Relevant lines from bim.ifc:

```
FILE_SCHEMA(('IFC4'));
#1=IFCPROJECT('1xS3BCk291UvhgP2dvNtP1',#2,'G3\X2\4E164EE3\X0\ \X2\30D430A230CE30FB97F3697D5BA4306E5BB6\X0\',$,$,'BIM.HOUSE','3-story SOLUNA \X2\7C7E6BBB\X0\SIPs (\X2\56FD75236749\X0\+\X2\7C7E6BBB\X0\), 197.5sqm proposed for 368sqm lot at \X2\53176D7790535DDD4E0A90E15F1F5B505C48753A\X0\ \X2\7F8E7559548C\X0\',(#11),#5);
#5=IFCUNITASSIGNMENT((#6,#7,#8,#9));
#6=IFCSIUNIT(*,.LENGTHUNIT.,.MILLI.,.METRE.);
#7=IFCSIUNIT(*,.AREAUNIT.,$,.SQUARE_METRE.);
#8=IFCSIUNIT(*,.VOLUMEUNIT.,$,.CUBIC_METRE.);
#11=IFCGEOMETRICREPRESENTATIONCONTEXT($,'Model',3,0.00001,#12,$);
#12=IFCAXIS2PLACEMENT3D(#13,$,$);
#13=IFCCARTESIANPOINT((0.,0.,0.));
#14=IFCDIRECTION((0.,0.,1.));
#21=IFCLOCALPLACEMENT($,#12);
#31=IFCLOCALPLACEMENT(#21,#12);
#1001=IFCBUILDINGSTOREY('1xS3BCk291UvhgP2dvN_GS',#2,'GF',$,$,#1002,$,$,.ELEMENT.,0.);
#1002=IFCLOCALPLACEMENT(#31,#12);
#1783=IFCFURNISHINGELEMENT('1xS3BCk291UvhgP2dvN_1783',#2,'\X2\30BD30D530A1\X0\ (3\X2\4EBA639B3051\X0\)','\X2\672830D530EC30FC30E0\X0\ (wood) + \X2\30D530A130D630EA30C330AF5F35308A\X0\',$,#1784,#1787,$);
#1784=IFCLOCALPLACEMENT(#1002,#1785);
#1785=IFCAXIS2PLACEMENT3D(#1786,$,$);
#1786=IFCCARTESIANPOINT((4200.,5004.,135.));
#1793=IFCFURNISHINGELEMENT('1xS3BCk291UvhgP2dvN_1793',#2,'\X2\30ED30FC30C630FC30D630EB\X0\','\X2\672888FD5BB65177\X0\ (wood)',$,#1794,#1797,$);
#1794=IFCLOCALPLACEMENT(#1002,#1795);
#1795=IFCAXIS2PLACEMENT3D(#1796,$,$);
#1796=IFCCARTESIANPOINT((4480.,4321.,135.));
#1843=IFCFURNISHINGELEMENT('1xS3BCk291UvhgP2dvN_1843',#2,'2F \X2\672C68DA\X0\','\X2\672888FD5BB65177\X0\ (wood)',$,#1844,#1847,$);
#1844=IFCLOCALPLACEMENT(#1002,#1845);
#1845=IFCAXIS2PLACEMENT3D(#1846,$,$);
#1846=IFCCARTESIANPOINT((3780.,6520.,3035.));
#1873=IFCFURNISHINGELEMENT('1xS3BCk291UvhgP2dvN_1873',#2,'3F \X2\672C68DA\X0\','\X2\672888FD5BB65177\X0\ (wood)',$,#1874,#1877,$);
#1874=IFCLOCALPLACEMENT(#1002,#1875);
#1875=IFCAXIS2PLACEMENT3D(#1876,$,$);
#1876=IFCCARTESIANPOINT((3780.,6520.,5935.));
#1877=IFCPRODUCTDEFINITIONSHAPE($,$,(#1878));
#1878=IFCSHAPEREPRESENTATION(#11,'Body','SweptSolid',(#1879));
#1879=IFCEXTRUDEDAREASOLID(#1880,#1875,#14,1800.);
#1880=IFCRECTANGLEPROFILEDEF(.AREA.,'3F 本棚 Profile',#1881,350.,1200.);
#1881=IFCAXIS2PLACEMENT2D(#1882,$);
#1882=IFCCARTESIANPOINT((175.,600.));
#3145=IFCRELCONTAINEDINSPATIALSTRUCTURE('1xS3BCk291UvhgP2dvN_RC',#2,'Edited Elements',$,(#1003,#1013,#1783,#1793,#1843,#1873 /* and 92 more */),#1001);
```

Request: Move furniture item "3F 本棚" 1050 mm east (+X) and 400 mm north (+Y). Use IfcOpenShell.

```python
import ifcopenshell
import ifcopenshell.api.geometry
import ifcopenshell.util.placement

model = ifcopenshell.open("bim.ifc")

item = model.by_guid("1xS3BCk291UvhgP2dvN_1873")
matrix = ifcopenshell.util.placement.get_local_placement(item.ObjectPlacement)
matrix[0, 3] += 1050.0
matrix[1, 3] += 400.0
ifcopenshell.api.geometry.edit_object_placement(model, product=item, matrix=matrix, is_si=False)

print(ifcopenshell.util.placement.get_local_placement(item.ObjectPlacement).round(3) + 0.0)

model.write("bim_updated.ifc")
```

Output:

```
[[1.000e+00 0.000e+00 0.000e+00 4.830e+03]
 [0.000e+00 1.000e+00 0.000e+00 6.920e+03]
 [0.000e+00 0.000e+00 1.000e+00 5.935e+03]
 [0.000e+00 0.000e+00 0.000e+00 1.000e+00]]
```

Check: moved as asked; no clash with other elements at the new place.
